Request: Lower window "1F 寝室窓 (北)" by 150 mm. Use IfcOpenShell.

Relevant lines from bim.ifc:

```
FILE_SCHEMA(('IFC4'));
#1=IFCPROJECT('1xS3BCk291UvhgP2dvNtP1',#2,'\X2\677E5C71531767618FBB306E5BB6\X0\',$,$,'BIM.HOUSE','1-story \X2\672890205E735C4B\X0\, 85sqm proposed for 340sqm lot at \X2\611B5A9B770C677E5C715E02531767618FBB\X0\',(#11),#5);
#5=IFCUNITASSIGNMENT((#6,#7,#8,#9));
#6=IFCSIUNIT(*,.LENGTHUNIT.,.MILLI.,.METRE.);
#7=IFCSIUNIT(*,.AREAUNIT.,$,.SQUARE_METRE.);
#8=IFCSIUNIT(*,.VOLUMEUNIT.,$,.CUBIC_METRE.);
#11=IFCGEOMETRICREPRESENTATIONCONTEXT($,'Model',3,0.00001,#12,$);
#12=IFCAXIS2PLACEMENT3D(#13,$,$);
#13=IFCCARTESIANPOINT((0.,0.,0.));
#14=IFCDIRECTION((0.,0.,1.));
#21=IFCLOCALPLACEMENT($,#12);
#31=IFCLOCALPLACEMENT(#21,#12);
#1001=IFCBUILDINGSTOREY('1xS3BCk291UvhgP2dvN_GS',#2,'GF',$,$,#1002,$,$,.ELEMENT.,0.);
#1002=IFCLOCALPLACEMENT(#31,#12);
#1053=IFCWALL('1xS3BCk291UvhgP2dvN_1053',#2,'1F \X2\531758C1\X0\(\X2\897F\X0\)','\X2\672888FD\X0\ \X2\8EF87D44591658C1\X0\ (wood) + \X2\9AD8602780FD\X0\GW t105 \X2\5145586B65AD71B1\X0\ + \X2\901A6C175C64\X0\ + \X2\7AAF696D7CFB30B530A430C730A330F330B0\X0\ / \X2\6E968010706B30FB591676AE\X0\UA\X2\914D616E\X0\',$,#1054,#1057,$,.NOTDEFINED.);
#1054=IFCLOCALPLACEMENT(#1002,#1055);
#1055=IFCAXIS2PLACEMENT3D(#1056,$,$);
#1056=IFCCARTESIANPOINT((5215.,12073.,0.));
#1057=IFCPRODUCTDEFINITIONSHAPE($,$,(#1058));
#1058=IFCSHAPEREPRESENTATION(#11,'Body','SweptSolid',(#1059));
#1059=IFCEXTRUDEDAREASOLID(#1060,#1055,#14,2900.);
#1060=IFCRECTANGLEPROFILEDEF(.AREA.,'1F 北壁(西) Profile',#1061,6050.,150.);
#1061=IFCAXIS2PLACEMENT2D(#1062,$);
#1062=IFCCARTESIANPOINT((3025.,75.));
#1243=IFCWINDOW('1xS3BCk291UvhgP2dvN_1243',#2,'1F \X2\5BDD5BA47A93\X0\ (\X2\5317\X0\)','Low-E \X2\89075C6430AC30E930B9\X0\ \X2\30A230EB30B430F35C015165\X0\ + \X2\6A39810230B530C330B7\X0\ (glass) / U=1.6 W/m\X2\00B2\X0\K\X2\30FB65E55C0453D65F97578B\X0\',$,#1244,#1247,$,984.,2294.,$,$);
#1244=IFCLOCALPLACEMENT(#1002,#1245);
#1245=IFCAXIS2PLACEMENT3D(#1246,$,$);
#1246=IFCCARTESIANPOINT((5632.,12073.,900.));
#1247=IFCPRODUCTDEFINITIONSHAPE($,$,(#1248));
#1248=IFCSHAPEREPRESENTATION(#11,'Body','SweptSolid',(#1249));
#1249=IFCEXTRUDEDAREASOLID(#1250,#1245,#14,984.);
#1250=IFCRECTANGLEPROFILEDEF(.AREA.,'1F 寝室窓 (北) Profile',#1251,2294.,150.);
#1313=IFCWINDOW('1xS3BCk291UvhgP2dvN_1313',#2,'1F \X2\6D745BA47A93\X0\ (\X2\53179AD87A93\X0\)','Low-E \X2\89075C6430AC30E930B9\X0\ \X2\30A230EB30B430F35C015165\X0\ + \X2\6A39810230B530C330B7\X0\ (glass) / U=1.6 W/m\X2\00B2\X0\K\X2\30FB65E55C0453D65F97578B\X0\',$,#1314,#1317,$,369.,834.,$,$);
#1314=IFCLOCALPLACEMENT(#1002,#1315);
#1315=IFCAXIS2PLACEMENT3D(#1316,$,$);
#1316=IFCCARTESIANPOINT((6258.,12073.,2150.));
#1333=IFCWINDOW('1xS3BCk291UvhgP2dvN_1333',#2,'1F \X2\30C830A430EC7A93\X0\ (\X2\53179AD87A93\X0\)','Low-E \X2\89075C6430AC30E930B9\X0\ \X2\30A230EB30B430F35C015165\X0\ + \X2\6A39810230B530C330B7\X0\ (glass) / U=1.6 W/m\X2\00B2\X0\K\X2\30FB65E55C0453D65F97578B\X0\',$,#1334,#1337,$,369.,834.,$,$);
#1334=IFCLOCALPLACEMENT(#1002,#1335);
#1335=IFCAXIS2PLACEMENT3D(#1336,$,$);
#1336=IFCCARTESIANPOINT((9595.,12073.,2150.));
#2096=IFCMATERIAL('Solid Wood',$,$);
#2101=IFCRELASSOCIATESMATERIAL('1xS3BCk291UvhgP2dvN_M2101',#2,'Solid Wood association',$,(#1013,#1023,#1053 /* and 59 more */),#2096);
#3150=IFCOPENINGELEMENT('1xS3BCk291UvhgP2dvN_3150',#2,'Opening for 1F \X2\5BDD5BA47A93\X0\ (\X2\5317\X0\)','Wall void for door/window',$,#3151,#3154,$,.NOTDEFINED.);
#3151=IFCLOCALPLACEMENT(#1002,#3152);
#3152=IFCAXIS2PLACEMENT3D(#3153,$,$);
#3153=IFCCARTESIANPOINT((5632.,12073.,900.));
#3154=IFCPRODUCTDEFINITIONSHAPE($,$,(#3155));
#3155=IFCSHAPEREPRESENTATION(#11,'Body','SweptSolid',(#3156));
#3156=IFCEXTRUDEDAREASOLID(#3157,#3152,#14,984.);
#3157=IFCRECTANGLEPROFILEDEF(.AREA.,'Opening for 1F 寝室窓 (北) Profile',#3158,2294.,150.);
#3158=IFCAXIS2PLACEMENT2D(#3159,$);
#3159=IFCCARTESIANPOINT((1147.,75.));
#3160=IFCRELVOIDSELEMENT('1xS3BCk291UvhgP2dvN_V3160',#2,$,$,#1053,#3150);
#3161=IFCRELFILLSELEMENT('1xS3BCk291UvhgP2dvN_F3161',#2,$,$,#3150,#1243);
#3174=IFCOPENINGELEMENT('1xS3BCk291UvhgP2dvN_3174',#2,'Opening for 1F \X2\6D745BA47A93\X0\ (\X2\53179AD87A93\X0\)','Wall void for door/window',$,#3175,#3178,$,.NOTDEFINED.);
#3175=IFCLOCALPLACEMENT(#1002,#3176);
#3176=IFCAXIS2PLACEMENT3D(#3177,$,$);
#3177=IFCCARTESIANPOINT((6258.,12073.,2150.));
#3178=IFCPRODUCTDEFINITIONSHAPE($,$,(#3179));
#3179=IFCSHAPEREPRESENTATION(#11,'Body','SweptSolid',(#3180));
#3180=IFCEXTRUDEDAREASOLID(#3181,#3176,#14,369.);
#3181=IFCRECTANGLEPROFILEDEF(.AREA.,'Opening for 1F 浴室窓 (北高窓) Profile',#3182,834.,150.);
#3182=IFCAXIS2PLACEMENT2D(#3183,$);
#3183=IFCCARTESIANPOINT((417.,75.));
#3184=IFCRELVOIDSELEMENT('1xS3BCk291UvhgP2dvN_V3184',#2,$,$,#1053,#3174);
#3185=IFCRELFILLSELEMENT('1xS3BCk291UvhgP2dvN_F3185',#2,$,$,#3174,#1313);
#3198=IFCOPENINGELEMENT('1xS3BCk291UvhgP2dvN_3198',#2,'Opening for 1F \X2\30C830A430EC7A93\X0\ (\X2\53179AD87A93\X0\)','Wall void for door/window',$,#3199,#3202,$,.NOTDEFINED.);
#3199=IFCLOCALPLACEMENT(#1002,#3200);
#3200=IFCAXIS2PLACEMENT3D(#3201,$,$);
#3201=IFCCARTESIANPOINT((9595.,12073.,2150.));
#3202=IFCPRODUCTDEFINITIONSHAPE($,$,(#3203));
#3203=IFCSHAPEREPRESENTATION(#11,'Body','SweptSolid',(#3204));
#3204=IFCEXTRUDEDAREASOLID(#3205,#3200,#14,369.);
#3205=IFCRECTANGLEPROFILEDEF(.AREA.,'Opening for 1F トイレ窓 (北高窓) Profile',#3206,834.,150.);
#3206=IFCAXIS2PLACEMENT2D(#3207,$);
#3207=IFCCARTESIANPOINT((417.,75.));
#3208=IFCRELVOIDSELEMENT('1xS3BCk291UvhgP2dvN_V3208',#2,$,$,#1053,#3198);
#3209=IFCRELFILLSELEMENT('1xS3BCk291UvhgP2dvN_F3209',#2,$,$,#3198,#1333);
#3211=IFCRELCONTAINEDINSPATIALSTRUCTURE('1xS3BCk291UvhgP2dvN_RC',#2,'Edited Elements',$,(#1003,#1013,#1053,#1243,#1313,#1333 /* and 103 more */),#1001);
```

```python
import numpy as np
import ifcopenshell
import ifcopenshell.api.geometry
import ifcopenshell.util.placement
import ifcopenshell.util.unit

model = ifcopenshell.open("bim.ifc")
unit_scale = ifcopenshell.util.unit.calculate_unit_scale(model)

window = model.by_guid("1xS3BCk291UvhgP2dvN_1243")
opening = window.FillsVoids[0].RelatingOpeningElement
dz = -150.0

shift = np.array([0.0, 0.0, dz])
# The window is not placed relative to its opening, so move both.
for product in (opening, window):
    matrix = ifcopenshell.util.placement.get_local_placement(product.ObjectPlacement)
    matrix[:3, 3] += shift
    ifcopenshell.api.geometry.edit_object_placement(model, product=product, matrix=matrix, is_si=False)

print(f"moved by {dz * unit_scale:+.3f} m")

model.write("bim_edited.ifc")
```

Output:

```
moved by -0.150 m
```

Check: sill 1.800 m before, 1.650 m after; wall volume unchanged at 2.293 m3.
